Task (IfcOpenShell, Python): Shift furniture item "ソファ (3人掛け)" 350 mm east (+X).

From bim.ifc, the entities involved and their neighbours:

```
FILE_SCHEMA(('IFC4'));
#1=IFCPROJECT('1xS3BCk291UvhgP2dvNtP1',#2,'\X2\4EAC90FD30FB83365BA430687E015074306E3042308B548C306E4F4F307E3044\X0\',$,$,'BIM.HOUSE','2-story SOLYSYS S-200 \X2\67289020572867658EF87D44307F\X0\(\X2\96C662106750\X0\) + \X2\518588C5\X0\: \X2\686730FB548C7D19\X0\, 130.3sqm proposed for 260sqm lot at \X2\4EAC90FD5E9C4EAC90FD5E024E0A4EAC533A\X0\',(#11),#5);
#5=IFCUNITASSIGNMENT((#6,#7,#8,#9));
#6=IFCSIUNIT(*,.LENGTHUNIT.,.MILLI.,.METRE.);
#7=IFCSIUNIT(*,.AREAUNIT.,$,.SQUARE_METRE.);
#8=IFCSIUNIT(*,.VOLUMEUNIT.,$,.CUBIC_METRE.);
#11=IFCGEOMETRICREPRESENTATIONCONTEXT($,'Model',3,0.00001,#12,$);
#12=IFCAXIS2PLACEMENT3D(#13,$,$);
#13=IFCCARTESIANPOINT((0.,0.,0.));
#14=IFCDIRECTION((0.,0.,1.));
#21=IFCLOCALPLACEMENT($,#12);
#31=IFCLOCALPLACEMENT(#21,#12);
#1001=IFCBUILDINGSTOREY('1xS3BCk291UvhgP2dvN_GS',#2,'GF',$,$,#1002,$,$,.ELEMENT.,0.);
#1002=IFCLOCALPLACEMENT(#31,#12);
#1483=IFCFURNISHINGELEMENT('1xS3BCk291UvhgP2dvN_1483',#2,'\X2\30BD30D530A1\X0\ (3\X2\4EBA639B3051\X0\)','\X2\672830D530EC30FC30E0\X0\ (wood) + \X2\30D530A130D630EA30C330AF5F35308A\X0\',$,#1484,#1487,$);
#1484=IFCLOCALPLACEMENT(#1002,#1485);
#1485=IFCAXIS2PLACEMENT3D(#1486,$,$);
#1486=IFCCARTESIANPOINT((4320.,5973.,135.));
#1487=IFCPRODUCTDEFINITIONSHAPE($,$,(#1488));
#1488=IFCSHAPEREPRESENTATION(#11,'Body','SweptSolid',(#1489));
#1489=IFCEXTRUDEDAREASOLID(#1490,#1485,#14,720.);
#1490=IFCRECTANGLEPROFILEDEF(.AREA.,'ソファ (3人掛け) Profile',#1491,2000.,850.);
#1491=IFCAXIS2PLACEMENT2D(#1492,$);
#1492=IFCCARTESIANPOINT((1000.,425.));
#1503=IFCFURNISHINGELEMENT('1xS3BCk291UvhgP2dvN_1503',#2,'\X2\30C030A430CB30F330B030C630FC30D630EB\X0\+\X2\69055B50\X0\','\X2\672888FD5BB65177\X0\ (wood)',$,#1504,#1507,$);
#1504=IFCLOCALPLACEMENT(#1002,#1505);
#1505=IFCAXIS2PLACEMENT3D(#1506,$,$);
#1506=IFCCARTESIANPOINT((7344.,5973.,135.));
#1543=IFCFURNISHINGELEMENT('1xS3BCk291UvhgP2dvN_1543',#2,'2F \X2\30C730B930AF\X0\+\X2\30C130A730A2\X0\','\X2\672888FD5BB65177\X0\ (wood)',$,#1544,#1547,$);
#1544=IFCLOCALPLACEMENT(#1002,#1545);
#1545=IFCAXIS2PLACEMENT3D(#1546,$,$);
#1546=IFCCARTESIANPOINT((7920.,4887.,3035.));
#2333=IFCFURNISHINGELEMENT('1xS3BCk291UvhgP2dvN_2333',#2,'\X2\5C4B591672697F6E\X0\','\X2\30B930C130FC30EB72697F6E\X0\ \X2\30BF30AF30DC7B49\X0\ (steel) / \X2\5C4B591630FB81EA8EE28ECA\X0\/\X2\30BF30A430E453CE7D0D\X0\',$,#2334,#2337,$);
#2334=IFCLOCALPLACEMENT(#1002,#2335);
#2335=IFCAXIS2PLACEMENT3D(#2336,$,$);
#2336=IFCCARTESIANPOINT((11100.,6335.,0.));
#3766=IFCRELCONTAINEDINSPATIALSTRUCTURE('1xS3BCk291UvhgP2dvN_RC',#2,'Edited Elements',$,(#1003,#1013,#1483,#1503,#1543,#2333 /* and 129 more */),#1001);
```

```python
import ifcopenshell
import ifcopenshell.api.geometry
import ifcopenshell.util.placement
import ifcopenshell.util.unit

model = ifcopenshell.open("bim.ifc")
unit_scale = ifcopenshell.util.unit.calculate_unit_scale(model)

item = model.by_guid("1xS3BCk291UvhgP2dvN_1483")
matrix = ifcopenshell.util.placement.get_local_placement(item.ObjectPlacement)
matrix[0, 3] += 0.35 / unit_scale
ifcopenshell.api.geometry.edit_object_placement(model, product=item, matrix=matrix, is_si=False)

print(ifcopenshell.util.placement.get_local_placement(item.ObjectPlacement).round(3) + 0.0)

model.write("bim-out.ifc")
```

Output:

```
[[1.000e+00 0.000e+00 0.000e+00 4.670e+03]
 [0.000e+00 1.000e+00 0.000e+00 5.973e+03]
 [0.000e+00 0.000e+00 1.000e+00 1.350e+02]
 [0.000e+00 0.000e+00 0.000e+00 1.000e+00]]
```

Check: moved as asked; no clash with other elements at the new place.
